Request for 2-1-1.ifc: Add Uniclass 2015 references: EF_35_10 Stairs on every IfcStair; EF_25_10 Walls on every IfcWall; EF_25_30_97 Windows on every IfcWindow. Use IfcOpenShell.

First a look at what the model holds.

```python
import ifcopenshell

model = ifcopenshell.open("2-1-1.ifc")
print(model.schema)
print("classifications:", [c.Name for c in model.by_type("IfcClassification")])
for ifc_class in ("IfcDoor", "IfcRoof", "IfcStair", "IfcWall", "IfcWindow"):
    print(ifc_class, len(model.by_type(ifc_class)))
```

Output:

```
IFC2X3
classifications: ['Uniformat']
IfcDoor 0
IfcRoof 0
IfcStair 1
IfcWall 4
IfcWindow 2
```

```python
import ifcopenshell
import ifcopenshell.api.classification

model = ifcopenshell.open("2-1-1.ifc")

# IFC2X3 requires Source and Edition and has no link from the project to the system.
system = model.create_entity("IfcClassification", Source="NBS", Edition="2015", Name="Uniclass 2015")

codes = {
    "IfcStair": ("EF_35_10", "Stairs"),
    "IfcWall": ("EF_25_10", "Walls"),
    "IfcWindow": ("EF_25_30_97", "Windows"),
}
for ifc_class, (code, name) in codes.items():
    products = model.by_type(ifc_class)
    ifcopenshell.api.classification.add_reference(
        model, products=products, classification=system, identification=code, name=name
    )
    print(code, len(products))

model.write("2-1-1_v2.ifc")
```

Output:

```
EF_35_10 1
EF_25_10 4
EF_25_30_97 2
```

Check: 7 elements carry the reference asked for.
